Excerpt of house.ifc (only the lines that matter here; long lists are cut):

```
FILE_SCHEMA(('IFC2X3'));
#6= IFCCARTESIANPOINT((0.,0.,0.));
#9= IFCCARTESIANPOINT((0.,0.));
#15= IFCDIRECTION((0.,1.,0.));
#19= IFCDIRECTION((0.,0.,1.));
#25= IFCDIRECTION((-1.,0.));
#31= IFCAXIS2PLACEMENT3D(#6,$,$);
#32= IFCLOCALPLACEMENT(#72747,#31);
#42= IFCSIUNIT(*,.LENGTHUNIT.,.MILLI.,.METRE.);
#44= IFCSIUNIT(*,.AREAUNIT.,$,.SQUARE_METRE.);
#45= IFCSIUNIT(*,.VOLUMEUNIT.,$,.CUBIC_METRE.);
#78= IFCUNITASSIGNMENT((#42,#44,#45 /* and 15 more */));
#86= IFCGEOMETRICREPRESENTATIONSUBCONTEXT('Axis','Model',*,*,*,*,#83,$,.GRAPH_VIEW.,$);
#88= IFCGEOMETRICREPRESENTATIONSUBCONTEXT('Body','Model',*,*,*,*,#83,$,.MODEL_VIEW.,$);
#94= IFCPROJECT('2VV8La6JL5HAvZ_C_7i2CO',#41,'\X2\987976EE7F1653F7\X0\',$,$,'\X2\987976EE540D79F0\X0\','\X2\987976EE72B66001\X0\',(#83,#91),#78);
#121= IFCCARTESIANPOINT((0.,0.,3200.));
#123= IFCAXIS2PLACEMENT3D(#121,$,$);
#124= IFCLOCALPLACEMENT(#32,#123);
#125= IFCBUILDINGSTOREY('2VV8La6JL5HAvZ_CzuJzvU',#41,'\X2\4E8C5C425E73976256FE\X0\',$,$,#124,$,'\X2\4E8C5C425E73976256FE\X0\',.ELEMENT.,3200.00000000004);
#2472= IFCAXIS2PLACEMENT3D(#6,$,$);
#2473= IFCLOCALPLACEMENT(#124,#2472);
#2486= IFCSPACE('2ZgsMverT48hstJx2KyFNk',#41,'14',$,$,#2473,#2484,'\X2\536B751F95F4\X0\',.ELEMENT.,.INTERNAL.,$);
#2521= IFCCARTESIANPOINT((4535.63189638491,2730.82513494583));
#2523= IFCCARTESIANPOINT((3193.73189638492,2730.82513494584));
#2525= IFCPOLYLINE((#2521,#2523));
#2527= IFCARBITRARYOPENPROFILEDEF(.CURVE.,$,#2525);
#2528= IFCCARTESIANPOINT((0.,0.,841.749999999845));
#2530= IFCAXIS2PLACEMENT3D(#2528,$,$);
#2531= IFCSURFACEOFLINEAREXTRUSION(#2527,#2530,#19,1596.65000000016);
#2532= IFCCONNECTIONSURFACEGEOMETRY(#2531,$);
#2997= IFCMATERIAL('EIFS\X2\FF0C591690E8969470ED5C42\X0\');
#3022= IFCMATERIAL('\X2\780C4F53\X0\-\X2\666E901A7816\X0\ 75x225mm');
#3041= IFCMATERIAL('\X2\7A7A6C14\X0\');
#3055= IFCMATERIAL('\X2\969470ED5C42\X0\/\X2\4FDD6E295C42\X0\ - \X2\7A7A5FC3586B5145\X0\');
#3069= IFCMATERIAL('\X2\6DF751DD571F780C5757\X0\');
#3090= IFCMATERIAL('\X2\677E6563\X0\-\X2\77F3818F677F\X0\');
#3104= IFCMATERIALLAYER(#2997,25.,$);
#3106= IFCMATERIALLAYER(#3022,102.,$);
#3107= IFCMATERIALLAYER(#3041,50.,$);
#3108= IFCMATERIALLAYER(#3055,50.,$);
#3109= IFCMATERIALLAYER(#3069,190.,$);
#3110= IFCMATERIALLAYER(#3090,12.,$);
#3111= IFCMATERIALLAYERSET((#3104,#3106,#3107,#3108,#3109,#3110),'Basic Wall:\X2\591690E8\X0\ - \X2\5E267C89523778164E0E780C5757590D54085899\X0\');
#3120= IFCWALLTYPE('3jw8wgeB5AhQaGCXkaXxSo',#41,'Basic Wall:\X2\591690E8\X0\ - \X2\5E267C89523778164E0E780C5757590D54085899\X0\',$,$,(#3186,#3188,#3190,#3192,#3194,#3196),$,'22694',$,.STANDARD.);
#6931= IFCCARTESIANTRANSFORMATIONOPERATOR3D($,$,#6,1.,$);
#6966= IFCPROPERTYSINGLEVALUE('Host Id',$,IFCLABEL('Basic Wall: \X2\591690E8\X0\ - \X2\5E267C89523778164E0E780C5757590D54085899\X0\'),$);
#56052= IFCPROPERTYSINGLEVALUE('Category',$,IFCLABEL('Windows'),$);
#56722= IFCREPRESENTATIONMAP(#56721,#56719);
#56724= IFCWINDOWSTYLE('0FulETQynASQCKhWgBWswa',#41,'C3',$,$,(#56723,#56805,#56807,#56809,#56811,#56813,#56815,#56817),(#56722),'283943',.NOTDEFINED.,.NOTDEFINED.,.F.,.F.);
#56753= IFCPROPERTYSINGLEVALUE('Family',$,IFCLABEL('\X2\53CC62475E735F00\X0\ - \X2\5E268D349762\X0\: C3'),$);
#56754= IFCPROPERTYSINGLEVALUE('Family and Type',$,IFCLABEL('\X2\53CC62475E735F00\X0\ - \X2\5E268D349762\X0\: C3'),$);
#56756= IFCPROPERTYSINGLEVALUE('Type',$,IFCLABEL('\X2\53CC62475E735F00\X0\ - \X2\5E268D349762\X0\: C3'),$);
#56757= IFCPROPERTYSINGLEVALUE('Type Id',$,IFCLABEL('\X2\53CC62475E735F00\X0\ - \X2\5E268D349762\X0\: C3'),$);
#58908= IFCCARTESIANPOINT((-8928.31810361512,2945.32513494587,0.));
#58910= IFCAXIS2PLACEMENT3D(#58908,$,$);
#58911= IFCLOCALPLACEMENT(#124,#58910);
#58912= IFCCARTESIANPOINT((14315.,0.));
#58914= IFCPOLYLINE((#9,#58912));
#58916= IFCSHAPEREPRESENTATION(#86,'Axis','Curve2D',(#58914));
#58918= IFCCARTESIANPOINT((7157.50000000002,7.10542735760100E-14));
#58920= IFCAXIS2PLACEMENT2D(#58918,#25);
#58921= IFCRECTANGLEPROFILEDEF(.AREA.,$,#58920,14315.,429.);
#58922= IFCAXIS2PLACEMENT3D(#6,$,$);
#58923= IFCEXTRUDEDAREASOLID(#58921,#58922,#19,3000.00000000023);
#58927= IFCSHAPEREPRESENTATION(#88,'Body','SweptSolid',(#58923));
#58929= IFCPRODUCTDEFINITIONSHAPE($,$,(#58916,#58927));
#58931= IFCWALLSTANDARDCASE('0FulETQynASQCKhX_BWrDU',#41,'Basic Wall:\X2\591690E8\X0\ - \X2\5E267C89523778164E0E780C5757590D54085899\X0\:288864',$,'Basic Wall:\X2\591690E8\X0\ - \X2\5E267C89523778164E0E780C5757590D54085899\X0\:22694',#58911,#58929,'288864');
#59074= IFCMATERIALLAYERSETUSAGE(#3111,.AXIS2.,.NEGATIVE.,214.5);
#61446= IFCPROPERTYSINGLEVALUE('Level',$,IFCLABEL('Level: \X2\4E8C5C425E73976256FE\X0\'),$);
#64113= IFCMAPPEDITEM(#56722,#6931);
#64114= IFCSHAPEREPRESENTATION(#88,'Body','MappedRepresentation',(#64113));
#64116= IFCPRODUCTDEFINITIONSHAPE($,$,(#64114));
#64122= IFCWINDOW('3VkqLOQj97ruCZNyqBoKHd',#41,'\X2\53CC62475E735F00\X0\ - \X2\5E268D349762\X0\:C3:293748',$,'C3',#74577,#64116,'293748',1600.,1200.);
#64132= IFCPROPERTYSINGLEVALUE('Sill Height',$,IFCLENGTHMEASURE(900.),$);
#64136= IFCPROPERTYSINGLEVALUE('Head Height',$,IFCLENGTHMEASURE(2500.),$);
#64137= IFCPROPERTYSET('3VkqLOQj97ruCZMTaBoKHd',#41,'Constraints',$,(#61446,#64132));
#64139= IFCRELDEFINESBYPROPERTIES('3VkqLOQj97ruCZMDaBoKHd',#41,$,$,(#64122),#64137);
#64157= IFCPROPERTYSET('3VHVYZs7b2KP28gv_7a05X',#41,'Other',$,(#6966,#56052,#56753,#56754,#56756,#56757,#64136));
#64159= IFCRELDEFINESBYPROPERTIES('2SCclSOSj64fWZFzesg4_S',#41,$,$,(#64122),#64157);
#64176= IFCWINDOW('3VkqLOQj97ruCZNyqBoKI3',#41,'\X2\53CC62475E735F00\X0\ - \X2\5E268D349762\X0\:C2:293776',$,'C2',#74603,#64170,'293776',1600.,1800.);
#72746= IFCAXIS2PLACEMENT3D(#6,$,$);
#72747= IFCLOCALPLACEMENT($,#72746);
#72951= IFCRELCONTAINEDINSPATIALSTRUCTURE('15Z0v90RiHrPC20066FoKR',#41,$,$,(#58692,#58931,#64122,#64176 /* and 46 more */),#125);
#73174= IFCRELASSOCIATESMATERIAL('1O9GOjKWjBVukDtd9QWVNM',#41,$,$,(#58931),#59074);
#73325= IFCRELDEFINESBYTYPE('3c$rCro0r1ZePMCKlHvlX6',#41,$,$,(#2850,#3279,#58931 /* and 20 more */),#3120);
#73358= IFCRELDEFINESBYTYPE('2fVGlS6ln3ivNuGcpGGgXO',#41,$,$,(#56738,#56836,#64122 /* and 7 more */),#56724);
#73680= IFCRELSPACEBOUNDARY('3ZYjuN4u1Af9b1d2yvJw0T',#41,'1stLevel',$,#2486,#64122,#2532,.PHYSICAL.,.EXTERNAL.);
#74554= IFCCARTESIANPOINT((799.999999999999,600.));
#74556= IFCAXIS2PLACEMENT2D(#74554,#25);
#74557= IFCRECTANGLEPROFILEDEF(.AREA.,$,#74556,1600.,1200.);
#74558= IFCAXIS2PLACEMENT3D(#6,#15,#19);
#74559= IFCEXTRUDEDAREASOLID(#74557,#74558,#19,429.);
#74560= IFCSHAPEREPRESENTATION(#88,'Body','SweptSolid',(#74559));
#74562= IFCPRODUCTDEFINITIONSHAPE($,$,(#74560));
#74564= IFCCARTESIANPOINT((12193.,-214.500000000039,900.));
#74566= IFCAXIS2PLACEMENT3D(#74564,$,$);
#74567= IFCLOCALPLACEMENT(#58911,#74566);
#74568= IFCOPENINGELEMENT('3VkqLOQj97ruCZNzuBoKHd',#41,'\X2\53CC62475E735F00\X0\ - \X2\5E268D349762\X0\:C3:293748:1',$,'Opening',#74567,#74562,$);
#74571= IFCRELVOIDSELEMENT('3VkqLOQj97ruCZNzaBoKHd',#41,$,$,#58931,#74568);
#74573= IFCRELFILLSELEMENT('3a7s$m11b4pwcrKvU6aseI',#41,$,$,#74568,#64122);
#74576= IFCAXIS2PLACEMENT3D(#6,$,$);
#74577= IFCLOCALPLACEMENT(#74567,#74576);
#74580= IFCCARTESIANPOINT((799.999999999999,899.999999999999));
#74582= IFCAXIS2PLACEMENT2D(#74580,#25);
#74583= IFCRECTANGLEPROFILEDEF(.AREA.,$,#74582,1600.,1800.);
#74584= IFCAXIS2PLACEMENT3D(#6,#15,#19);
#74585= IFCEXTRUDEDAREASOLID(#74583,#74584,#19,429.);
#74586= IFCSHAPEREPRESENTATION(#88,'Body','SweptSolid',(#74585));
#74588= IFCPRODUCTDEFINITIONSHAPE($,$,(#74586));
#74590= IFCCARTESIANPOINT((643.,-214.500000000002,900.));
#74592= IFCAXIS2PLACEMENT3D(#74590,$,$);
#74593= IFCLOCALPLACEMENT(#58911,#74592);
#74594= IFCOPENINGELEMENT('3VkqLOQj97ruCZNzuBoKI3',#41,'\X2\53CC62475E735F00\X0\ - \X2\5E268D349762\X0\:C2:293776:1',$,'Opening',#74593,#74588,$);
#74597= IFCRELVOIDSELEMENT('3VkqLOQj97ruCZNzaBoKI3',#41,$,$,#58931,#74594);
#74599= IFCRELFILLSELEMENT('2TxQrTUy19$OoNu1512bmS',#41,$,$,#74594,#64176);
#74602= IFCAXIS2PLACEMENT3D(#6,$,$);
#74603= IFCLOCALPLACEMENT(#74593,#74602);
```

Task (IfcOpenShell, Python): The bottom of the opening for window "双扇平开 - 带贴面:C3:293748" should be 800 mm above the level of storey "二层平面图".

```python
import numpy as np
import ifcopenshell
import ifcopenshell.api.geometry
import ifcopenshell.api.pset
import ifcopenshell.geom
import ifcopenshell.util.element
import ifcopenshell.util.placement
import ifcopenshell.util.shape
import ifcopenshell.util.unit

model = ifcopenshell.open("house.ifc")
unit_scale = ifcopenshell.util.unit.calculate_unit_scale(model)

window = model.by_id(64122)
opening = window.FillsVoids[0].RelatingOpeningElement
storey = ifcopenshell.util.element.get_container(window, ifc_class="IfcBuildingStorey")
level = ifcopenshell.util.placement.get_local_placement(storey.ObjectPlacement)[2, 3]

# The opening's origin need not be at the sill, so measure its lowest point.
shape = ifcopenshell.geom.create_shape(ifcopenshell.geom.settings(), opening)
bottom = ifcopenshell.util.shape.get_shape_bottom_elevation(shape, shape.geometry) / unit_scale
dz = level + 0.8 / unit_scale - bottom

shift = np.array([0.0, 0.0, dz])
# The window is placed relative to its opening, so it follows when the opening moves.
matrix = ifcopenshell.util.placement.get_local_placement(opening.ObjectPlacement)
matrix[:3, 3] += shift
ifcopenshell.api.geometry.edit_object_placement(
    model, product=opening, matrix=matrix, is_si=False, should_transform_children=True
)

# Space boundary surfaces are stored in each space's coordinates; move them too.
for rel in window.ProvidesBoundaries:
    if not rel.ConnectionGeometry:
        continue
    surface = rel.ConnectionGeometry.SurfaceOnRelatingElement
    space_matrix = ifcopenshell.util.placement.get_local_placement(rel.RelatingSpace.ObjectPlacement)
    point = np.array(surface.Position.Location.Coordinates) + space_matrix[:3, :3].T @ shift
    surface.Position = model.createIfcAxis2Placement3D(
        model.createIfcCartesianPoint(point.tolist()), surface.Position.Axis, surface.Position.RefDirection
    )

# Keep the stored heights in step.
pset = model.by_id(ifcopenshell.util.element.get_pset(window, "Constraints", should_inherit=False)["id"])
ifcopenshell.api.pset.edit_pset(model, pset=pset, properties={
    "Sill Height": model.create_entity("IfcLengthMeasure", ifcopenshell.util.element.get_pset(window, "Constraints", "Sill Height") + dz),
})
pset = model.by_id(ifcopenshell.util.element.get_pset(window, "Other", should_inherit=False)["id"])
ifcopenshell.api.pset.edit_pset(model, pset=pset, properties={
    "Head Height": model.create_entity("IfcLengthMeasure", ifcopenshell.util.element.get_pset(window, "Other", "Head Height") + dz),
})

print(f"moved by {dz * unit_scale:+.3f} m")

model.write("house_edited.ifc")
```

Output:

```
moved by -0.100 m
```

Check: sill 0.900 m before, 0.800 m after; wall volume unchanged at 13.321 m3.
